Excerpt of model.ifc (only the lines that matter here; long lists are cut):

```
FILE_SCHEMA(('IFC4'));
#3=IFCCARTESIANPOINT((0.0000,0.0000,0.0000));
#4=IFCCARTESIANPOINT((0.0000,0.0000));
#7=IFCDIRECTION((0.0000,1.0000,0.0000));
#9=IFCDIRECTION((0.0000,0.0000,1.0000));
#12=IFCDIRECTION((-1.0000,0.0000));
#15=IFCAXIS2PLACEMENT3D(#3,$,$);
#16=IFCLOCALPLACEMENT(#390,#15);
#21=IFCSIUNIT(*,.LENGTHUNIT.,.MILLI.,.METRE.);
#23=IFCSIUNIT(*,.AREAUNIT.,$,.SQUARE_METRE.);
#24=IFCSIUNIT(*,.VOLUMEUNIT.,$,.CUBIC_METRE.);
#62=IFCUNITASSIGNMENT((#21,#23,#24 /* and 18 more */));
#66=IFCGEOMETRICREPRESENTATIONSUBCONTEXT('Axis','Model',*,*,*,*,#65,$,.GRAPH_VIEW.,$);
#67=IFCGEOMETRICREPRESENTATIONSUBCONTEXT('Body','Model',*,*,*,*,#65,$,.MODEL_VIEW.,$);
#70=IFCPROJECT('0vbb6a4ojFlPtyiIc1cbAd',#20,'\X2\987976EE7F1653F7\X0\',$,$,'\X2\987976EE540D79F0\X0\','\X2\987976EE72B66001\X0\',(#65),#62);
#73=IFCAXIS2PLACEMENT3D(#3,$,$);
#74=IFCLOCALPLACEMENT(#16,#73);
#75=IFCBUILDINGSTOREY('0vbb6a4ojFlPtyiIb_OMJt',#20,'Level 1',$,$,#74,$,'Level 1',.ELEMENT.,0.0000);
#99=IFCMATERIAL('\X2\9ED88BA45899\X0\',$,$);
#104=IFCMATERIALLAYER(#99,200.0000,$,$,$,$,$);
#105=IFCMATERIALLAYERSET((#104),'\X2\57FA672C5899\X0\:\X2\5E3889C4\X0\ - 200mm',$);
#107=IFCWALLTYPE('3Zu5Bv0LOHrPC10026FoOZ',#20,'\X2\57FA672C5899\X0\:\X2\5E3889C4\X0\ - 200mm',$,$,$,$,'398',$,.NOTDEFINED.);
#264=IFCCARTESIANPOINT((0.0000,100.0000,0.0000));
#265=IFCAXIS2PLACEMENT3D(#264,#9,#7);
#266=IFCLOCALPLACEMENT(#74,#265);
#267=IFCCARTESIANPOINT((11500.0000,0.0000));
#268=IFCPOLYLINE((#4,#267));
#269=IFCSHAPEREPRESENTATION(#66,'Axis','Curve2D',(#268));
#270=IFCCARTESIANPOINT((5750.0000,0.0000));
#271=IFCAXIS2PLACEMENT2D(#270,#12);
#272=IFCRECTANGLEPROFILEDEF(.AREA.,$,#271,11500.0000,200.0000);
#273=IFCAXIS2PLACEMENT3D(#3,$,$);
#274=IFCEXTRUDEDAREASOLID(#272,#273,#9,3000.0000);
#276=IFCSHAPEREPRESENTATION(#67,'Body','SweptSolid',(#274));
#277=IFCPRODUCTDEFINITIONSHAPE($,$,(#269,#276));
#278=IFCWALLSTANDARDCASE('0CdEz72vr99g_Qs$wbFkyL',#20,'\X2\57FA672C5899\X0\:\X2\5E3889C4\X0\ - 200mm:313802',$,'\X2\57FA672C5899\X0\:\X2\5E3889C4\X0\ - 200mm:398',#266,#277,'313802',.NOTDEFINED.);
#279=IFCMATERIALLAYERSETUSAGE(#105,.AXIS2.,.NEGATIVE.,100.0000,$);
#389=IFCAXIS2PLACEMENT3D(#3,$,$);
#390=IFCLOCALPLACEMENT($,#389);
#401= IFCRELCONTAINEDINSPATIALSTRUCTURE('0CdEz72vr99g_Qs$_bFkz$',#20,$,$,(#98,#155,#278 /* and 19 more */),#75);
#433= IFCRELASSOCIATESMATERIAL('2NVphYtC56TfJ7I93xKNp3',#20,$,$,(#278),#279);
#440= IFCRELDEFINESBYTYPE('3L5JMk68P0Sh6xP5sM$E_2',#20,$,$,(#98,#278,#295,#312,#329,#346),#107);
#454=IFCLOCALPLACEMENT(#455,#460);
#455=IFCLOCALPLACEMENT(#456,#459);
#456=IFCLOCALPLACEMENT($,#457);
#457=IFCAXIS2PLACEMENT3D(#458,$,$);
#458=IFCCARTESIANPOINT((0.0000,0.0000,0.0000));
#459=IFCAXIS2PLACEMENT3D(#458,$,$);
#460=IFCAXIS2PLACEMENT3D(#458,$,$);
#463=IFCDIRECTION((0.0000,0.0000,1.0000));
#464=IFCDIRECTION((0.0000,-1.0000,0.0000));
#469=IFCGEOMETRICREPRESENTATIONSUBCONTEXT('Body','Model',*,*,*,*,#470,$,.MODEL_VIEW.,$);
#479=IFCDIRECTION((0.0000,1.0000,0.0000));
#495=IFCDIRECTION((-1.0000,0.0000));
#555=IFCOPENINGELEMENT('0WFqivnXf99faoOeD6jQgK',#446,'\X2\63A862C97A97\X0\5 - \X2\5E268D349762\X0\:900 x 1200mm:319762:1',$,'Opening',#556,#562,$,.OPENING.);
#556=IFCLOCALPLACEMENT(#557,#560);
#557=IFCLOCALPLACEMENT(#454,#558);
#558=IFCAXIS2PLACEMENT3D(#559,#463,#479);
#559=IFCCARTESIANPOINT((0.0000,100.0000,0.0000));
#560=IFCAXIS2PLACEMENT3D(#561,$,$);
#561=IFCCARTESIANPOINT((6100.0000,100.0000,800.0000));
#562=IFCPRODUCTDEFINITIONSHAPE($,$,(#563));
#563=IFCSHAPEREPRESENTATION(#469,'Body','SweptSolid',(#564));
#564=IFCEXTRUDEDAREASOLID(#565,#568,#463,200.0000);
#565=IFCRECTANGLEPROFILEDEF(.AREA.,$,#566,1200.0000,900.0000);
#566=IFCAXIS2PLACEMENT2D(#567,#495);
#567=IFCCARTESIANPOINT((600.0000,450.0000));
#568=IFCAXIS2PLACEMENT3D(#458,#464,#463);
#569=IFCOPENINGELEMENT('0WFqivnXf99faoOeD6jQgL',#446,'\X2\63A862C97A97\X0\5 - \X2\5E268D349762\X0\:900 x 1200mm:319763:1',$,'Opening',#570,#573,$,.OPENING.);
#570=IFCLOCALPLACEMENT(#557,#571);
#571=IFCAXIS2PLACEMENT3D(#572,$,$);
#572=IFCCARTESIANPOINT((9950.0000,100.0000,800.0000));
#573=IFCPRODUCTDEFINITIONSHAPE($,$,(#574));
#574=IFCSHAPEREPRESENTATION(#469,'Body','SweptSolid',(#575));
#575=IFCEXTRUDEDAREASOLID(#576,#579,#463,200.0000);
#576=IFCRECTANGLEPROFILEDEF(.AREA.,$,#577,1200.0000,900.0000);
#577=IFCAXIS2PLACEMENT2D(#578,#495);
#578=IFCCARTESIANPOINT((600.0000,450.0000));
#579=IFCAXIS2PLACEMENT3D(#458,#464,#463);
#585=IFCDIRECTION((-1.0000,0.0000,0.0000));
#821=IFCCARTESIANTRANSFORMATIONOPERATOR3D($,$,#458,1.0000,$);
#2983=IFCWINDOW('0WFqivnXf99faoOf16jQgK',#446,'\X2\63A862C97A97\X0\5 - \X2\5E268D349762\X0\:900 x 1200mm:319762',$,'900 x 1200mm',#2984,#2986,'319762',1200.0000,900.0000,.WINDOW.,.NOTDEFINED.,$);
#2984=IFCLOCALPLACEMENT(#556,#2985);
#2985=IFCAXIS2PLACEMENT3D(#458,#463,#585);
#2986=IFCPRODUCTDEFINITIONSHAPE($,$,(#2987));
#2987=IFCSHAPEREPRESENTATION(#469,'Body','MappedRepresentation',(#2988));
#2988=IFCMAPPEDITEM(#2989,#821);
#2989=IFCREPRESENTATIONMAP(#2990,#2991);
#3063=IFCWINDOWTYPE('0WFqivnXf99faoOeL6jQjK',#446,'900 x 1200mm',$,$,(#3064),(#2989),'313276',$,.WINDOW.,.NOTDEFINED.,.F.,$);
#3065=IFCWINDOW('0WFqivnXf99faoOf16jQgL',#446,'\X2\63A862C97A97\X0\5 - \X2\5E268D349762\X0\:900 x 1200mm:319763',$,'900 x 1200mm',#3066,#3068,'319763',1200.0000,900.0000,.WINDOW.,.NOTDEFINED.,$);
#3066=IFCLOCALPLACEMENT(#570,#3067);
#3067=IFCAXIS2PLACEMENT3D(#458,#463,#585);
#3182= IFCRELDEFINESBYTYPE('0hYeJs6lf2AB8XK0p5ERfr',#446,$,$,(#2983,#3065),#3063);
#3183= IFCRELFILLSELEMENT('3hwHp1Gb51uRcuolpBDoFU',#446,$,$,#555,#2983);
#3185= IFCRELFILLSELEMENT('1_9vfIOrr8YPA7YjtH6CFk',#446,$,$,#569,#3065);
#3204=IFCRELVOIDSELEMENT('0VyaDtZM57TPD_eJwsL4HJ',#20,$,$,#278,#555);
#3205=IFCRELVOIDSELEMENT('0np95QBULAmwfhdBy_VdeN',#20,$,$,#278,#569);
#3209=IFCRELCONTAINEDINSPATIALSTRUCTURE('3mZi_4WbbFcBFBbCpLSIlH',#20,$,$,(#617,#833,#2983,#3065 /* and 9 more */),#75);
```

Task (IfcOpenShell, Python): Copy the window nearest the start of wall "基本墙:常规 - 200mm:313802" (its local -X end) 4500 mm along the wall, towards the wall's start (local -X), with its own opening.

```python
import ifcopenshell
import ifcopenshell.api.feature
import ifcopenshell.api.geometry
import ifcopenshell.api.root
import ifcopenshell.geom
import ifcopenshell.util.element
import ifcopenshell.util.placement
import ifcopenshell.util.shape

model = ifcopenshell.open("model.ifc")
settings = ifcopenshell.geom.settings()


def volume(element):
    """Net volume in cubic metres, openings subtracted."""
    shape = ifcopenshell.geom.create_shape(settings, element)
    return ifcopenshell.util.shape.get_volume(shape.geometry)


def reuse_history(source, copy):
    """copy_class also copies each property set's owner history, people and application; keep the originals."""
    for rel in copy.IsDefinedBy:
        if rel.is_a("IfcRelDefinesByProperties") and (history := rel.RelatingPropertyDefinition.OwnerHistory):
            rel.RelatingPropertyDefinition.OwnerHistory = source.OwnerHistory
            ifcopenshell.util.element.remove_deep2(model, history)


window = model.by_id(2983)
opening = window.FillsVoids[0].RelatingOpeningElement
wall = opening.VoidsElements[0].RelatingBuildingElement
before = volume(wall)
shift = ifcopenshell.util.placement.get_local_placement(wall.ObjectPlacement)[:3, 0] * -4500.0

# copy_class copies the void relationship, type, container and properties, but no geometry.
new_opening = ifcopenshell.api.root.copy_class(model, product=opening)
new_opening.Representation = ifcopenshell.util.element.copy_deep(
    model, opening.Representation, exclude=["IfcGeometricRepresentationContext", "IfcRepresentationMap"]
)
new_opening.Name = "推拉窗5 - 带贴面:900 x 1200mm"
new_window = ifcopenshell.api.root.copy_class(model, product=window)
new_window.Representation = ifcopenshell.util.element.copy_deep(
    model, window.Representation, exclude=["IfcGeometricRepresentationContext", "IfcRepresentationMap"]
)
new_window.Name = "推拉窗5 - 带贴面:900 x 1200mm"
new_window.Tag = None
reuse_history(window, new_window)
ifcopenshell.api.feature.add_filling(model, opening=new_opening, element=new_window)

for old, new in ((opening, new_opening), (window, new_window)):
    matrix = ifcopenshell.util.placement.get_local_placement(old.ObjectPlacement)
    matrix[:3, 3] += shift
    ifcopenshell.api.geometry.edit_object_placement(model, product=new, matrix=matrix, is_si=False)

after = volume(wall)

print(f"wall volume {before:.3f} -> {after:.3f} m3")

model.write("model_edited.ifc")
```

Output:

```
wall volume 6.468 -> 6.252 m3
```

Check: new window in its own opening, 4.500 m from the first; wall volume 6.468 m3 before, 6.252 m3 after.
